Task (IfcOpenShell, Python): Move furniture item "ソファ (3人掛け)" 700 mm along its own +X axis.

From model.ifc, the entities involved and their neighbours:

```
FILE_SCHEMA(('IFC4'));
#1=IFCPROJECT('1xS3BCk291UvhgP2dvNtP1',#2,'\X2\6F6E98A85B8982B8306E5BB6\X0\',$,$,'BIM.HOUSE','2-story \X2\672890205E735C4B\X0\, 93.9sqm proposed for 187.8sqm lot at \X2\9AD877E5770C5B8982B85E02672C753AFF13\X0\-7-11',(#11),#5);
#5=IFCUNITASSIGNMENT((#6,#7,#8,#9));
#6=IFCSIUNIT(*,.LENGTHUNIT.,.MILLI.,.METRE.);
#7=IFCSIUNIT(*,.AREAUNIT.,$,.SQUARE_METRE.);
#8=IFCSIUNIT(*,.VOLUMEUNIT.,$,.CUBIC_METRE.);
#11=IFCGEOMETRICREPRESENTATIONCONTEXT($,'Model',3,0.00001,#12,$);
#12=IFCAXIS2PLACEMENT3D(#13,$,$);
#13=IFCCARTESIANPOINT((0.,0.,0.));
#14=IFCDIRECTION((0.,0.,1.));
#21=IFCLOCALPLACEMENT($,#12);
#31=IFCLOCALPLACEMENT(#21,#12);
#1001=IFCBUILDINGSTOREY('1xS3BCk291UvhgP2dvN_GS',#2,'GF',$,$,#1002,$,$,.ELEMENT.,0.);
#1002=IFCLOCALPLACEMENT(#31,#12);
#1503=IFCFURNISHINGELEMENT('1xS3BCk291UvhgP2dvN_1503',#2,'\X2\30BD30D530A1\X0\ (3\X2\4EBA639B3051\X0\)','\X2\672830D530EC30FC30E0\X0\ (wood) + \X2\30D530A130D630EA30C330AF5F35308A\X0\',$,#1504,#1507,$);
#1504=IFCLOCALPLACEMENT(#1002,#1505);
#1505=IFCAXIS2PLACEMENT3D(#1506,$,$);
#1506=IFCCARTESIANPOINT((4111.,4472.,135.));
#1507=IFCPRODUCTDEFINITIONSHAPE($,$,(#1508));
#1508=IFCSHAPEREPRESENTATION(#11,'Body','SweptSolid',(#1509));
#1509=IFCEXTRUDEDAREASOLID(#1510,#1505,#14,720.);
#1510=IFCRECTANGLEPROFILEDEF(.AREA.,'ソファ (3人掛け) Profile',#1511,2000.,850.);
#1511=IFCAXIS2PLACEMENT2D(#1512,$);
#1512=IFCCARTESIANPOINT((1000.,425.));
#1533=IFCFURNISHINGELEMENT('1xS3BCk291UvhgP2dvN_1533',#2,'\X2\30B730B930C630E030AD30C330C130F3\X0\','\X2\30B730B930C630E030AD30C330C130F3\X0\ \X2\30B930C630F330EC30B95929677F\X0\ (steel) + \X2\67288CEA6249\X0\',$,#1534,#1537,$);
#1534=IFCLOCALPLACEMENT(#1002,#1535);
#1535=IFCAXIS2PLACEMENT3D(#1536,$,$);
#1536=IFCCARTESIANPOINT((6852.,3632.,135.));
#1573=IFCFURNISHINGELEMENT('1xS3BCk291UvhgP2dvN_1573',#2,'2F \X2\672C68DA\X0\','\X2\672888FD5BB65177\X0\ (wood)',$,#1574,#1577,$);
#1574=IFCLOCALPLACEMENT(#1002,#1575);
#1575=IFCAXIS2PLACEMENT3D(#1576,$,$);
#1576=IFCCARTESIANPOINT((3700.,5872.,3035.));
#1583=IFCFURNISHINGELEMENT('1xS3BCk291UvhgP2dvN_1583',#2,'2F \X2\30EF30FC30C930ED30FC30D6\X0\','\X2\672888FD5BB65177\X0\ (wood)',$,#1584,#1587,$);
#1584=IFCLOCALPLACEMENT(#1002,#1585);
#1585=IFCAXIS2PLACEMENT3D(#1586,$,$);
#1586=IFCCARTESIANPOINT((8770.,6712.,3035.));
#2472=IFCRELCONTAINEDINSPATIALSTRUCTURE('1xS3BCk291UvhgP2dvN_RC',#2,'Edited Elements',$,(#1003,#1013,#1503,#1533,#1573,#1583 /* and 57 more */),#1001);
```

```python
import ifcopenshell
import ifcopenshell.api.geometry
import ifcopenshell.util.placement
import ifcopenshell.util.unit

model = ifcopenshell.open("model.ifc")
unit_scale = ifcopenshell.util.unit.calculate_unit_scale(model)

item = model.by_guid("1xS3BCk291UvhgP2dvN_1503")
matrix = ifcopenshell.util.placement.get_local_placement(item.ObjectPlacement)
matrix[:3, 3] += matrix[:3, 0] * 0.7 / unit_scale
ifcopenshell.api.geometry.edit_object_placement(model, product=item, matrix=matrix, is_si=False)

print(ifcopenshell.util.placement.get_local_placement(item.ObjectPlacement).round(3) + 0.0)

model.write("model_v2.ifc")
```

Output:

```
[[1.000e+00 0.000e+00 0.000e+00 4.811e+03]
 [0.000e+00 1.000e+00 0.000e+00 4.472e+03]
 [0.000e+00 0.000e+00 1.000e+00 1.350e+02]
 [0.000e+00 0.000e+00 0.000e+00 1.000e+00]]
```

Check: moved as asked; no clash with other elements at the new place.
